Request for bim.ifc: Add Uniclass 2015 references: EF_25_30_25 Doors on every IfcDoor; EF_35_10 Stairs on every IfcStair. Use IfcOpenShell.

First a look at what the model holds.

```python
import ifcopenshell

model = ifcopenshell.open("bim.ifc")
print(model.schema)
print("classifications:", [c.Name for c in model.by_type("IfcClassification")])
for ifc_class in ("IfcDoor", "IfcRoof", "IfcStair", "IfcWall", "IfcWindow"):
    print(ifc_class, len(model.by_type(ifc_class)))
```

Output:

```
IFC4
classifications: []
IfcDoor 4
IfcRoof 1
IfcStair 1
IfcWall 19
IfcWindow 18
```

```python
import ifcopenshell
import ifcopenshell.api.classification

model = ifcopenshell.open("bim.ifc")

system = ifcopenshell.api.classification.add_classification(model, classification="Uniclass 2015")

codes = {
    "IfcDoor": ("EF_25_30_25", "Doors"),
    "IfcStair": ("EF_35_10", "Stairs"),
}
for ifc_class, (code, name) in codes.items():
    products = model.by_type(ifc_class)
    ifcopenshell.api.classification.add_reference(
        model, products=products, classification=system, identification=code, name=name
    )
    print(code, len(products))

model.write("bim_v2.ifc")
```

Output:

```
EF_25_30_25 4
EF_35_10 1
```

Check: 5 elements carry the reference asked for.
